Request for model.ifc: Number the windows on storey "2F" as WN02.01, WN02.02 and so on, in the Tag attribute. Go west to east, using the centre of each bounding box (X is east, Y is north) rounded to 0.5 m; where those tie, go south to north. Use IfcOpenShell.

First a look at what the model holds.

```python
import ifcopenshell
import ifcopenshell.util.element
import ifcopenshell.util.placement

model = ifcopenshell.open("model.ifc")
print(model.schema)
storey = next(s for s in model.by_type("IfcBuildingStorey") if s.Name == "2F")
windows = [e for e in ifcopenshell.util.element.get_decomposition(storey) if e.is_a("IfcWindow")]
for e in sorted(windows, key=lambda e: e.id()):
    origin = ifcopenshell.util.placement.get_local_placement(e.ObjectPlacement)[:3, 3]
    print(e.id(), e.Tag, e.Name, origin.round(2) + 0.0, sep=" | ")
```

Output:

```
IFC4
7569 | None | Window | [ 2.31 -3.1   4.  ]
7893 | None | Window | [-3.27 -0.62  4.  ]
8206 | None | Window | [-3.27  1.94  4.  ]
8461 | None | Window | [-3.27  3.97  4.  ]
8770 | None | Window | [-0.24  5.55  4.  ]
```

```python
import ifcopenshell
import ifcopenshell.geom
import ifcopenshell.util.element
import ifcopenshell.util.shape

model = ifcopenshell.open("model.ifc")
settings = ifcopenshell.geom.settings()
settings.set("use-world-coords", True)


def centre(element):
    shape = ifcopenshell.geom.create_shape(settings, element)
    return ifcopenshell.util.shape.get_bbox_centroid(shape.geometry)


storey = next(s for s in model.by_type("IfcBuildingStorey") if s.Name == "2F")
windows = [e for e in ifcopenshell.util.element.get_decomposition(storey) if e.is_a("IfcWindow")]

# Insertion points can sit at a corner or the storey origin, so sort by the geometry (in metres).
centres = {e: centre(e) for e in windows}
windows.sort(key=lambda e: (round(centres[e][0] / 0.5), centres[e][1]))

for i, e in enumerate(windows, start=1):
    number = f"WN02.{i:02d}"
    e.Tag = number
    print(e.id(), number)

model.write("model-out.ifc")
```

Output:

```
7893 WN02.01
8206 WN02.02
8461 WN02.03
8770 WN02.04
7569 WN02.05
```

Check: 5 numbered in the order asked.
